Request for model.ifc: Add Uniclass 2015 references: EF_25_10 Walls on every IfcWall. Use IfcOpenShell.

First a look at what the model holds.

```python
import ifcopenshell

model = ifcopenshell.open("model.ifc")
print(model.schema)
print("classifications:", [c.Name for c in model.by_type("IfcClassification")])
for ifc_class in ("IfcDoor", "IfcRoof", "IfcStair", "IfcWall", "IfcWindow"):
    print(ifc_class, len(model.by_type(ifc_class)))
```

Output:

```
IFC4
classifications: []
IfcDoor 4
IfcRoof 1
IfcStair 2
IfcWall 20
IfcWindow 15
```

```python
import ifcopenshell
import ifcopenshell.api.classification

model = ifcopenshell.open("model.ifc")

system = ifcopenshell.api.classification.add_classification(model, classification="Uniclass 2015")

codes = {
    "IfcWall": ("EF_25_10", "Walls"),
}
for ifc_class, (code, name) in codes.items():
    products = model.by_type(ifc_class)
    ifcopenshell.api.classification.add_reference(
        model, products=products, classification=system, identification=code, name=name
    )
    print(code, len(products))

model.write("model_edited.ifc")
```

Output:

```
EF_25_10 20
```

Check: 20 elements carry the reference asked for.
